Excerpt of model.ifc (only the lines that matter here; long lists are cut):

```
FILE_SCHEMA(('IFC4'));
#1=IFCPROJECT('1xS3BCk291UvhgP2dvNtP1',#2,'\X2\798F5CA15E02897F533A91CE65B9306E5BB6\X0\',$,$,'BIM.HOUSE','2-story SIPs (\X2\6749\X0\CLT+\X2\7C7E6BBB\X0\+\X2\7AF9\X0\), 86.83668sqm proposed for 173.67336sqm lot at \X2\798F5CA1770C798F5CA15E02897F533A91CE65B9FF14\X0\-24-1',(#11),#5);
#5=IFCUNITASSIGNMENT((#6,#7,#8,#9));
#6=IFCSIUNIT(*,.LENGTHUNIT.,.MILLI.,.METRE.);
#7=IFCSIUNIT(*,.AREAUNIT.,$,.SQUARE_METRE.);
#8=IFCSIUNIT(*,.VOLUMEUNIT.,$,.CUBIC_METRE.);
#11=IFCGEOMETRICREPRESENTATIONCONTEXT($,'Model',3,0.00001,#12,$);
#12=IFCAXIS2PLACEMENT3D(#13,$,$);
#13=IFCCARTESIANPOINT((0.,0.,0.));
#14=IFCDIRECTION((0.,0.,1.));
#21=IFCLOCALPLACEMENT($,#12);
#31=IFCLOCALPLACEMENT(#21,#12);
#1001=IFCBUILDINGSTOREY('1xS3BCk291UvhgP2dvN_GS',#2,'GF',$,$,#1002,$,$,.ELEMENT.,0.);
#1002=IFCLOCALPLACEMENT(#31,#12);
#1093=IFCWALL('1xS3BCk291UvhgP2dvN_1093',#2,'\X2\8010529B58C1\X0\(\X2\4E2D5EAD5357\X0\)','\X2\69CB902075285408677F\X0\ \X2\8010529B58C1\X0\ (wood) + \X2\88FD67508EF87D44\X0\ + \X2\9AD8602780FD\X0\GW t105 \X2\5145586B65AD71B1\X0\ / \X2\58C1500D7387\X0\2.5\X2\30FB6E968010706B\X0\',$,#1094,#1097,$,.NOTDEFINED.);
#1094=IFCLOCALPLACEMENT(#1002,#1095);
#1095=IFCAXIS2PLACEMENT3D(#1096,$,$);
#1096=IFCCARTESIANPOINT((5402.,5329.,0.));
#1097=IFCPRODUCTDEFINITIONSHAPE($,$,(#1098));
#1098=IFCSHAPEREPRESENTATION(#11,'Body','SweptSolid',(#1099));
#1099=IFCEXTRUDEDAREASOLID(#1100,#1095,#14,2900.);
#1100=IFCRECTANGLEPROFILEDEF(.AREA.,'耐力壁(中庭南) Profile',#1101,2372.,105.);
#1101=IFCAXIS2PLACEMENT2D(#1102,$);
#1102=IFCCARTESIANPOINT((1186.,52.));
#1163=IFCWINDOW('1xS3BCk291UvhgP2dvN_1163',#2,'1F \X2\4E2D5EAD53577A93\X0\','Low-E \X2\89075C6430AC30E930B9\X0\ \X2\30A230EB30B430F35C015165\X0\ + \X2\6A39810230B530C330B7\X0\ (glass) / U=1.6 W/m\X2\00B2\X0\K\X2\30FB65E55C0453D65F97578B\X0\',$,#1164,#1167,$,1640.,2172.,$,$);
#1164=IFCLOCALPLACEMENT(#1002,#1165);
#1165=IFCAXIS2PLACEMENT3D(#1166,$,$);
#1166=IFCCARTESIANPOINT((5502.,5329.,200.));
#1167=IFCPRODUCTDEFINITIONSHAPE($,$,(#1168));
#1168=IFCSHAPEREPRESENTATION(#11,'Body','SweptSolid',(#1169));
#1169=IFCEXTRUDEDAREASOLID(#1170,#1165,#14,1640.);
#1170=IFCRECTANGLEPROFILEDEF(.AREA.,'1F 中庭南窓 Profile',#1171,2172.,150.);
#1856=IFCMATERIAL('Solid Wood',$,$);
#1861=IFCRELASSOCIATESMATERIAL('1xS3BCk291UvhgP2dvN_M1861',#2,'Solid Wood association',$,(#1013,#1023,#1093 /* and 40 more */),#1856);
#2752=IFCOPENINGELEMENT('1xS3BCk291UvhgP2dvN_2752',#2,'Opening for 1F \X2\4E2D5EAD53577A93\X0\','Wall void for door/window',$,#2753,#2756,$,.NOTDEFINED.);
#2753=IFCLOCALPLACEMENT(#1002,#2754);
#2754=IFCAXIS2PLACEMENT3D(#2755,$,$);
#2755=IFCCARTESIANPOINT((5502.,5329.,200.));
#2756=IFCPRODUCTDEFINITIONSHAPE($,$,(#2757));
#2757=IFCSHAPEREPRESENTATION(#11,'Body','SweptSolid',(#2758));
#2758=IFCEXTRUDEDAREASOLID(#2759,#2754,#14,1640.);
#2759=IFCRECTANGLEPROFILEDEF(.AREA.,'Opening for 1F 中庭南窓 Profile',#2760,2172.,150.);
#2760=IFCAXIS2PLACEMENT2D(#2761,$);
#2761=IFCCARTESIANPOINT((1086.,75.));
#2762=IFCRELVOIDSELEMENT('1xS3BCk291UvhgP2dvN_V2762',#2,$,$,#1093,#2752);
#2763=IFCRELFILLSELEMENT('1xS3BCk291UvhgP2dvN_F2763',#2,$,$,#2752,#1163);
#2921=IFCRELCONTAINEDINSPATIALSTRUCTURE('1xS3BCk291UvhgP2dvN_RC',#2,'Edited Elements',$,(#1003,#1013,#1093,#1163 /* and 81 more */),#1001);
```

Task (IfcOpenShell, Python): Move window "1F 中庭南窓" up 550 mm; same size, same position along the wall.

```python
import numpy as np
import ifcopenshell
import ifcopenshell.api.geometry
import ifcopenshell.util.placement
import ifcopenshell.util.unit

model = ifcopenshell.open("model.ifc")
unit_scale = ifcopenshell.util.unit.calculate_unit_scale(model)

window = model.by_guid("1xS3BCk291UvhgP2dvN_1163")
opening = window.FillsVoids[0].RelatingOpeningElement
dz = 0.55 / unit_scale

shift = np.array([0.0, 0.0, dz])
# The window is not placed relative to its opening, so move both.
for product in (opening, window):
    matrix = ifcopenshell.util.placement.get_local_placement(product.ObjectPlacement)
    matrix[:3, 3] += shift
    ifcopenshell.api.geometry.edit_object_placement(model, product=product, matrix=matrix, is_si=False)

print(f"moved by {dz * unit_scale:+.3f} m")

model.write("model_edited.ifc")
```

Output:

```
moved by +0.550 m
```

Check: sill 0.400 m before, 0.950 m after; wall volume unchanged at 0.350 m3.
